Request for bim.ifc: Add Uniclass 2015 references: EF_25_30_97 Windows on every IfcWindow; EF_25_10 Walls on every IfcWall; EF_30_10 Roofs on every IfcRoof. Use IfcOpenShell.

First a look at what the model holds.

```python
import ifcopenshell

model = ifcopenshell.open("bim.ifc")
print(model.schema)
print("classifications:", [c.Name for c in model.by_type("IfcClassification")])
for ifc_class in ("IfcDoor", "IfcRoof", "IfcStair", "IfcWall", "IfcWindow"):
    print(ifc_class, len(model.by_type(ifc_class)))
```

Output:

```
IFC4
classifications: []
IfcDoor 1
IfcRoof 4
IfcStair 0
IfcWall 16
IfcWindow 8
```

```python
import ifcopenshell
import ifcopenshell.api.classification

model = ifcopenshell.open("bim.ifc")

system = ifcopenshell.api.classification.add_classification(model, classification="Uniclass 2015")

codes = {
    "IfcWindow": ("EF_25_30_97", "Windows"),
    "IfcWall": ("EF_25_10", "Walls"),
    "IfcRoof": ("EF_30_10", "Roofs"),
}
for ifc_class, (code, name) in codes.items():
    products = model.by_type(ifc_class)
    ifcopenshell.api.classification.add_reference(
        model, products=products, classification=system, identification=code, name=name
    )
    print(code, len(products))

model.write("bim_updated.ifc")
```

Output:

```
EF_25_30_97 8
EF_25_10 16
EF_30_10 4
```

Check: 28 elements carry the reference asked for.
